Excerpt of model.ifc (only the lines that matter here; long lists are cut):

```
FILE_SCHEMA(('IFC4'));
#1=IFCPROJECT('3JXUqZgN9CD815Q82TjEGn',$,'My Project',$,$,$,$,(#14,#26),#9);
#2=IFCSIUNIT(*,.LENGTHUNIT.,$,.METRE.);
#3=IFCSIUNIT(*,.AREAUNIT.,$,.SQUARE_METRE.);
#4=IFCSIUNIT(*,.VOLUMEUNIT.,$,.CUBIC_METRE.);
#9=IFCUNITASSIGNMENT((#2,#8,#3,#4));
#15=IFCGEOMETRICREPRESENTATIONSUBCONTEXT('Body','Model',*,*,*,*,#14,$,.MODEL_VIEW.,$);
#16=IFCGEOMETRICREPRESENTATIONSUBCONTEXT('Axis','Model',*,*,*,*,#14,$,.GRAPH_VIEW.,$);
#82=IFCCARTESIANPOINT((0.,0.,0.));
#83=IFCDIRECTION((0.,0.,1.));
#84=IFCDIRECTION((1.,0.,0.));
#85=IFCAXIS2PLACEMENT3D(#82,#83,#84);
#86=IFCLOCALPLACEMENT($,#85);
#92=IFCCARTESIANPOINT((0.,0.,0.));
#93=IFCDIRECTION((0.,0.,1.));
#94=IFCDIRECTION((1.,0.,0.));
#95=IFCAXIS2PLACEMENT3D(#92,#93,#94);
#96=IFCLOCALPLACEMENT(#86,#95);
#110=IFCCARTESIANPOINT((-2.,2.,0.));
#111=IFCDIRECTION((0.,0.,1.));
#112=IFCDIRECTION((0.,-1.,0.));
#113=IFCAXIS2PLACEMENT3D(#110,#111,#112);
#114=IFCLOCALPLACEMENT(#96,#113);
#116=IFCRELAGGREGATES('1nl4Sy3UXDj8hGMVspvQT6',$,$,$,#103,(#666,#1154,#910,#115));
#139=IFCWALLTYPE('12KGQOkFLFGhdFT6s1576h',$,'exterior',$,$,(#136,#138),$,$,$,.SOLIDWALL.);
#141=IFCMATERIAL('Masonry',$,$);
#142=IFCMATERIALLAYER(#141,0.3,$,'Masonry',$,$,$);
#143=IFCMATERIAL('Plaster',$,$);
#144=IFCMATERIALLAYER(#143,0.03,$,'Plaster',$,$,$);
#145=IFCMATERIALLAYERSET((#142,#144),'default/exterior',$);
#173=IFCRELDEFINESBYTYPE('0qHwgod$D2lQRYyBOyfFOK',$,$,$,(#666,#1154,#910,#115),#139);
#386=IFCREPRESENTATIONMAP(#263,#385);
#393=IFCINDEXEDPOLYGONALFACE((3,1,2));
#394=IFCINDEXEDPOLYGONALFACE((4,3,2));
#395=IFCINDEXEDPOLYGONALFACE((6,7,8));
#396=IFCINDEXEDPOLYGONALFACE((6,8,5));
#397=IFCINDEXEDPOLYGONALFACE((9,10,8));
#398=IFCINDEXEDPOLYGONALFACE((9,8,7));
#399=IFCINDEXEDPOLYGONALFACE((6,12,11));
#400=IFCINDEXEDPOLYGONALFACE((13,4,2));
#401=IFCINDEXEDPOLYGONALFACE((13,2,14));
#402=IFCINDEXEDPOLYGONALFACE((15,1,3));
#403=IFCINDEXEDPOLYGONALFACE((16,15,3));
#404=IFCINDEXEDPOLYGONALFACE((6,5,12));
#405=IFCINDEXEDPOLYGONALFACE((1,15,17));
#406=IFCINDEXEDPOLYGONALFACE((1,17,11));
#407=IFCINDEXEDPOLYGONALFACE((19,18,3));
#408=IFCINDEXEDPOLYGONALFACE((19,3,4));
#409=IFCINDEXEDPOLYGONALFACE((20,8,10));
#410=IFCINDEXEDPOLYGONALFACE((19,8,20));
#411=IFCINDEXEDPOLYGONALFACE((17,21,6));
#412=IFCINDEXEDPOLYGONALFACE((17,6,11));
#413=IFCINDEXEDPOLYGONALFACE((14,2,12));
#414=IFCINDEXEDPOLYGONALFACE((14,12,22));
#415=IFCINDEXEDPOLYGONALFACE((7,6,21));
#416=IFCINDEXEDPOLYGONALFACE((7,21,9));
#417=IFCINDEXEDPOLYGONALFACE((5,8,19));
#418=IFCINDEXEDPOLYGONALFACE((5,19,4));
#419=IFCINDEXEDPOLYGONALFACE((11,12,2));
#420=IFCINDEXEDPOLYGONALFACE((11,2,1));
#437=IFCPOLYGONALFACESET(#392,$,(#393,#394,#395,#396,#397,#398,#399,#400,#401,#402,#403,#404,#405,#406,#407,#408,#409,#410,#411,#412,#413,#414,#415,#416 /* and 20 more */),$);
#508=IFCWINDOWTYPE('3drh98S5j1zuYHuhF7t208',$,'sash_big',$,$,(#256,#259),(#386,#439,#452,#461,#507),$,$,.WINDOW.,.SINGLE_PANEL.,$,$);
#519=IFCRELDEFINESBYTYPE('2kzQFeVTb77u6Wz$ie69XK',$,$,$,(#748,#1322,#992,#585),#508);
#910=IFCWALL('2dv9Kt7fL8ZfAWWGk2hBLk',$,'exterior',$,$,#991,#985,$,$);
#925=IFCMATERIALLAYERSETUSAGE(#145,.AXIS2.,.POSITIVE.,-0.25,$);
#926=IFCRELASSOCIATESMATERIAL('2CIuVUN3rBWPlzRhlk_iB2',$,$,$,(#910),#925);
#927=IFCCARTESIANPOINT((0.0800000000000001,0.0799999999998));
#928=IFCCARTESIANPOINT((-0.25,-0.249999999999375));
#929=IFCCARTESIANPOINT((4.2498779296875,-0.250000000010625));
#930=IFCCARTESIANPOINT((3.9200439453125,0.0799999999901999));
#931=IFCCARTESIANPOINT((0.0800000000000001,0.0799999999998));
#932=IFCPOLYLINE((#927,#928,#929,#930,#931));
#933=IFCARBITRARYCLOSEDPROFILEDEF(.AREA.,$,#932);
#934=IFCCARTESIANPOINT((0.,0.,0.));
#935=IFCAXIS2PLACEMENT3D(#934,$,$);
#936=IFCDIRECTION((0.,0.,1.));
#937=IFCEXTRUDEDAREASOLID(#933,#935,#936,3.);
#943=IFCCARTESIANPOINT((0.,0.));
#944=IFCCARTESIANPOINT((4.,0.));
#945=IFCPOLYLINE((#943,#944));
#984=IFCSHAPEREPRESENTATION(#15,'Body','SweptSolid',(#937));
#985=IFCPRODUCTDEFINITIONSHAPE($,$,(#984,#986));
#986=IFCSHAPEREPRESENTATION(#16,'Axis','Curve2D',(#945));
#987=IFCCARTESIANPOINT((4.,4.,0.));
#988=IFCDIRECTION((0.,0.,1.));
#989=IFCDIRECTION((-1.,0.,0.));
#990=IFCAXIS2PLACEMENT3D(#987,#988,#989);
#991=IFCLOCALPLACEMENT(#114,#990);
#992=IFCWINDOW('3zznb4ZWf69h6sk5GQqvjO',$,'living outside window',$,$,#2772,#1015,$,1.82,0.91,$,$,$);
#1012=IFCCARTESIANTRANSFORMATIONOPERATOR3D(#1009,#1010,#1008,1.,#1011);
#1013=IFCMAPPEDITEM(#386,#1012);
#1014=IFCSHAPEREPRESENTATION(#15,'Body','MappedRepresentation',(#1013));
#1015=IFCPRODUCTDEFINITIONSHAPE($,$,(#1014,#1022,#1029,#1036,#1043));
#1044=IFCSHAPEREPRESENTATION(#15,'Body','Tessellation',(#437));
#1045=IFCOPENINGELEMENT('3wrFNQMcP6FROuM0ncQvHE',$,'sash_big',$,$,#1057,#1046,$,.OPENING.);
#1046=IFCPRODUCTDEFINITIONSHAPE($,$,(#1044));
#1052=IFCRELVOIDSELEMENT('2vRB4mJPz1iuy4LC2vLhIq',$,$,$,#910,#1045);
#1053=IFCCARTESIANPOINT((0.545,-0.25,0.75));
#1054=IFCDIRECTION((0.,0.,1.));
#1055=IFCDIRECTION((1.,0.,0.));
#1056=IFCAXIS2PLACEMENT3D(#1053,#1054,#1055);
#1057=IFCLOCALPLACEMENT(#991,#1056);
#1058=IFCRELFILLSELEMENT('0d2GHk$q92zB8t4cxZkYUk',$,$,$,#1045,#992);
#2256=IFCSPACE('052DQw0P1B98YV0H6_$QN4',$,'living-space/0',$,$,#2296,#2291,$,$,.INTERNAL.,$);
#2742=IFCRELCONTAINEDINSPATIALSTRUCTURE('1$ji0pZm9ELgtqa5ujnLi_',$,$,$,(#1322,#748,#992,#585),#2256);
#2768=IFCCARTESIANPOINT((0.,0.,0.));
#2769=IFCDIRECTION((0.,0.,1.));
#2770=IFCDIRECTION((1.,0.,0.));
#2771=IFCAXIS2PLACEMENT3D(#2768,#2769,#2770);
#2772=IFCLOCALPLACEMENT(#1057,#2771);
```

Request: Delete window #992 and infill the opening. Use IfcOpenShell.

```python
import ifcopenshell
import ifcopenshell.api.feature
import ifcopenshell.api.root
import ifcopenshell.geom
import ifcopenshell.util.shape

model = ifcopenshell.open("model.ifc")
settings = ifcopenshell.geom.settings()


def volume(element):
    """Net volume in cubic metres, openings subtracted."""
    shape = ifcopenshell.geom.create_shape(settings, element)
    return ifcopenshell.util.shape.get_volume(shape.geometry)


window = model.by_id(992)
opening = window.FillsVoids[0].RelatingOpeningElement
wall = opening.VoidsElements[0].RelatingBuildingElement
before = volume(wall)

ifcopenshell.api.root.remove_product(model, product=window)
ifcopenshell.api.feature.remove_feature(model, feature=opening)

after = volume(wall)

print(f"wall volume {before:.3f} -> {after:.3f} m3")

model.write("model_updated.ifc")
```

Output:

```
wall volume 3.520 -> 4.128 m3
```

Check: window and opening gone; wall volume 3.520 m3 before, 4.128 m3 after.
